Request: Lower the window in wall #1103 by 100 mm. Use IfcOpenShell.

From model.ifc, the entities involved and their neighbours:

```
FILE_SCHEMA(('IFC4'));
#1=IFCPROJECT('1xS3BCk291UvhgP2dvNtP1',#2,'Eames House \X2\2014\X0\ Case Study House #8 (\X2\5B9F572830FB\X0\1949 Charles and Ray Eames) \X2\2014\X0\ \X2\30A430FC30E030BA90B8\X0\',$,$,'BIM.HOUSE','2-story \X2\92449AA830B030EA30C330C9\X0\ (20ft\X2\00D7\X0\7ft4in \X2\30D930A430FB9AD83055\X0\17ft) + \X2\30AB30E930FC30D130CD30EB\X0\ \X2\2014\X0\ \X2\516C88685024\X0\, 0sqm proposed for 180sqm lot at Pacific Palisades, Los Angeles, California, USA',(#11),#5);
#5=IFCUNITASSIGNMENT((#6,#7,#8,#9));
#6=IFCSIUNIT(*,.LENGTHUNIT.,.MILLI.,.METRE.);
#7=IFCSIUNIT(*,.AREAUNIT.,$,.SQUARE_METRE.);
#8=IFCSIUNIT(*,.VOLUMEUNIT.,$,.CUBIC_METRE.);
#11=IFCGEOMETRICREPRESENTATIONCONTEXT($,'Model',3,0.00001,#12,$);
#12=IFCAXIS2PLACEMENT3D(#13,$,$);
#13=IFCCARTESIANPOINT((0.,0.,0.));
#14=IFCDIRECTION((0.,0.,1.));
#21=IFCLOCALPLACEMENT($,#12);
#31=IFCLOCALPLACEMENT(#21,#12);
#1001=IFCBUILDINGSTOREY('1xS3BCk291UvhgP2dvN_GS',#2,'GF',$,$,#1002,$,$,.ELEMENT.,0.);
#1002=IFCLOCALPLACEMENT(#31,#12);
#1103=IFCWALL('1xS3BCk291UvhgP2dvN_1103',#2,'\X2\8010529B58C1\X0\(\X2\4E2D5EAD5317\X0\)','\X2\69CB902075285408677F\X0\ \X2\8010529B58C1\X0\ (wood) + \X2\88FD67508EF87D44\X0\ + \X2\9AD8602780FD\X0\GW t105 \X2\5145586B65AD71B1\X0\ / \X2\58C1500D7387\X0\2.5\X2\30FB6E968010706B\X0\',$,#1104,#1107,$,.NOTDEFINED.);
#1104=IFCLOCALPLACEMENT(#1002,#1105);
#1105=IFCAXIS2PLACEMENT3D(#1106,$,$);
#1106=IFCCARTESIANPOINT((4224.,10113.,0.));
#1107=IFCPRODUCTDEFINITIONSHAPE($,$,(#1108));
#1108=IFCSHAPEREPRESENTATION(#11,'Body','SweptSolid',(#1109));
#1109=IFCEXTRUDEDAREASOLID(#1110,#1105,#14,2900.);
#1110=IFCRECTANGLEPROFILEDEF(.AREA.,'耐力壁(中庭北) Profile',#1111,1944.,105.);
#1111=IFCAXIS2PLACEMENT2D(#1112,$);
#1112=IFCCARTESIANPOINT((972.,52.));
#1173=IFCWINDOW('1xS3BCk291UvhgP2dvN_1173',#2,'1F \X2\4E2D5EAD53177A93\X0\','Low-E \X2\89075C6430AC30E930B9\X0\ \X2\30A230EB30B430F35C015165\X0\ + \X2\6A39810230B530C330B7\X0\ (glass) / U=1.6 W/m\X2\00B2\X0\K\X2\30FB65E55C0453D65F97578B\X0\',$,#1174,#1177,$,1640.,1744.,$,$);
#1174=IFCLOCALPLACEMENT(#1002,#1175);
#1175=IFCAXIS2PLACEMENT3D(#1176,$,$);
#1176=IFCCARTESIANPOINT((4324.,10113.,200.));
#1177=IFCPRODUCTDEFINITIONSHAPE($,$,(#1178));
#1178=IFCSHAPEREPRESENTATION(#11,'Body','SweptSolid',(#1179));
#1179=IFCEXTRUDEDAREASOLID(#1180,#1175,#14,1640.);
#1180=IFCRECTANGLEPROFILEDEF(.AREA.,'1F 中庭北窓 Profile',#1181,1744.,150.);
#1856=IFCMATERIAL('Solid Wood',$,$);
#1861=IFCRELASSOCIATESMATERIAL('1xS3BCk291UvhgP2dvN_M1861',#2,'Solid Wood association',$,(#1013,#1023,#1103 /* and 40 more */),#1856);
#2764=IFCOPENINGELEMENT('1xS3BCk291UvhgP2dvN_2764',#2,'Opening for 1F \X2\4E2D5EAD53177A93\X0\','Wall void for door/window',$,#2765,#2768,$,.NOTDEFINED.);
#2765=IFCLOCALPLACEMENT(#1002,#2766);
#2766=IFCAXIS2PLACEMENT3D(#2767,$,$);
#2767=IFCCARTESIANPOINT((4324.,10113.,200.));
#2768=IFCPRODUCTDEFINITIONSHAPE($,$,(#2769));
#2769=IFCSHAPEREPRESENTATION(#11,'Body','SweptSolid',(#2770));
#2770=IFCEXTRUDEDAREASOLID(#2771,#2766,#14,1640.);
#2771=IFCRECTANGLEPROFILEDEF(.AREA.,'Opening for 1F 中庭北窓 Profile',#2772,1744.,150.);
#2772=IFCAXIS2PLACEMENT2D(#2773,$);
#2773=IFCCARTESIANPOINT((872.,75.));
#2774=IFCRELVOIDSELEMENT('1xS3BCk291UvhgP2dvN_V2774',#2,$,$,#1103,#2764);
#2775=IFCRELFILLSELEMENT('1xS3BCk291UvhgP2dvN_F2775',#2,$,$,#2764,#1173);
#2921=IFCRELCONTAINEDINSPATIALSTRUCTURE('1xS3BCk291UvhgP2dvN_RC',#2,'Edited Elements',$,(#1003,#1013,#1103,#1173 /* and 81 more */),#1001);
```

```python
import numpy as np
import ifcopenshell
import ifcopenshell.api.geometry
import ifcopenshell.util.placement
import ifcopenshell.util.unit

model = ifcopenshell.open("model.ifc")
unit_scale = ifcopenshell.util.unit.calculate_unit_scale(model)

window = model.by_guid("1xS3BCk291UvhgP2dvN_1173")
opening = window.FillsVoids[0].RelatingOpeningElement
dz = -0.1 / unit_scale

shift = np.array([0.0, 0.0, dz])
# The window is not placed relative to its opening, so move both.
for product in (opening, window):
    matrix = ifcopenshell.util.placement.get_local_placement(product.ObjectPlacement)
    matrix[:3, 3] += shift
    ifcopenshell.api.geometry.edit_object_placement(model, product=product, matrix=matrix, is_si=False)

print(f"moved by {dz * unit_scale:+.3f} m")

model.write("model_edited.ifc")
```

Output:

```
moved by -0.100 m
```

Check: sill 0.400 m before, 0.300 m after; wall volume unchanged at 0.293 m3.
